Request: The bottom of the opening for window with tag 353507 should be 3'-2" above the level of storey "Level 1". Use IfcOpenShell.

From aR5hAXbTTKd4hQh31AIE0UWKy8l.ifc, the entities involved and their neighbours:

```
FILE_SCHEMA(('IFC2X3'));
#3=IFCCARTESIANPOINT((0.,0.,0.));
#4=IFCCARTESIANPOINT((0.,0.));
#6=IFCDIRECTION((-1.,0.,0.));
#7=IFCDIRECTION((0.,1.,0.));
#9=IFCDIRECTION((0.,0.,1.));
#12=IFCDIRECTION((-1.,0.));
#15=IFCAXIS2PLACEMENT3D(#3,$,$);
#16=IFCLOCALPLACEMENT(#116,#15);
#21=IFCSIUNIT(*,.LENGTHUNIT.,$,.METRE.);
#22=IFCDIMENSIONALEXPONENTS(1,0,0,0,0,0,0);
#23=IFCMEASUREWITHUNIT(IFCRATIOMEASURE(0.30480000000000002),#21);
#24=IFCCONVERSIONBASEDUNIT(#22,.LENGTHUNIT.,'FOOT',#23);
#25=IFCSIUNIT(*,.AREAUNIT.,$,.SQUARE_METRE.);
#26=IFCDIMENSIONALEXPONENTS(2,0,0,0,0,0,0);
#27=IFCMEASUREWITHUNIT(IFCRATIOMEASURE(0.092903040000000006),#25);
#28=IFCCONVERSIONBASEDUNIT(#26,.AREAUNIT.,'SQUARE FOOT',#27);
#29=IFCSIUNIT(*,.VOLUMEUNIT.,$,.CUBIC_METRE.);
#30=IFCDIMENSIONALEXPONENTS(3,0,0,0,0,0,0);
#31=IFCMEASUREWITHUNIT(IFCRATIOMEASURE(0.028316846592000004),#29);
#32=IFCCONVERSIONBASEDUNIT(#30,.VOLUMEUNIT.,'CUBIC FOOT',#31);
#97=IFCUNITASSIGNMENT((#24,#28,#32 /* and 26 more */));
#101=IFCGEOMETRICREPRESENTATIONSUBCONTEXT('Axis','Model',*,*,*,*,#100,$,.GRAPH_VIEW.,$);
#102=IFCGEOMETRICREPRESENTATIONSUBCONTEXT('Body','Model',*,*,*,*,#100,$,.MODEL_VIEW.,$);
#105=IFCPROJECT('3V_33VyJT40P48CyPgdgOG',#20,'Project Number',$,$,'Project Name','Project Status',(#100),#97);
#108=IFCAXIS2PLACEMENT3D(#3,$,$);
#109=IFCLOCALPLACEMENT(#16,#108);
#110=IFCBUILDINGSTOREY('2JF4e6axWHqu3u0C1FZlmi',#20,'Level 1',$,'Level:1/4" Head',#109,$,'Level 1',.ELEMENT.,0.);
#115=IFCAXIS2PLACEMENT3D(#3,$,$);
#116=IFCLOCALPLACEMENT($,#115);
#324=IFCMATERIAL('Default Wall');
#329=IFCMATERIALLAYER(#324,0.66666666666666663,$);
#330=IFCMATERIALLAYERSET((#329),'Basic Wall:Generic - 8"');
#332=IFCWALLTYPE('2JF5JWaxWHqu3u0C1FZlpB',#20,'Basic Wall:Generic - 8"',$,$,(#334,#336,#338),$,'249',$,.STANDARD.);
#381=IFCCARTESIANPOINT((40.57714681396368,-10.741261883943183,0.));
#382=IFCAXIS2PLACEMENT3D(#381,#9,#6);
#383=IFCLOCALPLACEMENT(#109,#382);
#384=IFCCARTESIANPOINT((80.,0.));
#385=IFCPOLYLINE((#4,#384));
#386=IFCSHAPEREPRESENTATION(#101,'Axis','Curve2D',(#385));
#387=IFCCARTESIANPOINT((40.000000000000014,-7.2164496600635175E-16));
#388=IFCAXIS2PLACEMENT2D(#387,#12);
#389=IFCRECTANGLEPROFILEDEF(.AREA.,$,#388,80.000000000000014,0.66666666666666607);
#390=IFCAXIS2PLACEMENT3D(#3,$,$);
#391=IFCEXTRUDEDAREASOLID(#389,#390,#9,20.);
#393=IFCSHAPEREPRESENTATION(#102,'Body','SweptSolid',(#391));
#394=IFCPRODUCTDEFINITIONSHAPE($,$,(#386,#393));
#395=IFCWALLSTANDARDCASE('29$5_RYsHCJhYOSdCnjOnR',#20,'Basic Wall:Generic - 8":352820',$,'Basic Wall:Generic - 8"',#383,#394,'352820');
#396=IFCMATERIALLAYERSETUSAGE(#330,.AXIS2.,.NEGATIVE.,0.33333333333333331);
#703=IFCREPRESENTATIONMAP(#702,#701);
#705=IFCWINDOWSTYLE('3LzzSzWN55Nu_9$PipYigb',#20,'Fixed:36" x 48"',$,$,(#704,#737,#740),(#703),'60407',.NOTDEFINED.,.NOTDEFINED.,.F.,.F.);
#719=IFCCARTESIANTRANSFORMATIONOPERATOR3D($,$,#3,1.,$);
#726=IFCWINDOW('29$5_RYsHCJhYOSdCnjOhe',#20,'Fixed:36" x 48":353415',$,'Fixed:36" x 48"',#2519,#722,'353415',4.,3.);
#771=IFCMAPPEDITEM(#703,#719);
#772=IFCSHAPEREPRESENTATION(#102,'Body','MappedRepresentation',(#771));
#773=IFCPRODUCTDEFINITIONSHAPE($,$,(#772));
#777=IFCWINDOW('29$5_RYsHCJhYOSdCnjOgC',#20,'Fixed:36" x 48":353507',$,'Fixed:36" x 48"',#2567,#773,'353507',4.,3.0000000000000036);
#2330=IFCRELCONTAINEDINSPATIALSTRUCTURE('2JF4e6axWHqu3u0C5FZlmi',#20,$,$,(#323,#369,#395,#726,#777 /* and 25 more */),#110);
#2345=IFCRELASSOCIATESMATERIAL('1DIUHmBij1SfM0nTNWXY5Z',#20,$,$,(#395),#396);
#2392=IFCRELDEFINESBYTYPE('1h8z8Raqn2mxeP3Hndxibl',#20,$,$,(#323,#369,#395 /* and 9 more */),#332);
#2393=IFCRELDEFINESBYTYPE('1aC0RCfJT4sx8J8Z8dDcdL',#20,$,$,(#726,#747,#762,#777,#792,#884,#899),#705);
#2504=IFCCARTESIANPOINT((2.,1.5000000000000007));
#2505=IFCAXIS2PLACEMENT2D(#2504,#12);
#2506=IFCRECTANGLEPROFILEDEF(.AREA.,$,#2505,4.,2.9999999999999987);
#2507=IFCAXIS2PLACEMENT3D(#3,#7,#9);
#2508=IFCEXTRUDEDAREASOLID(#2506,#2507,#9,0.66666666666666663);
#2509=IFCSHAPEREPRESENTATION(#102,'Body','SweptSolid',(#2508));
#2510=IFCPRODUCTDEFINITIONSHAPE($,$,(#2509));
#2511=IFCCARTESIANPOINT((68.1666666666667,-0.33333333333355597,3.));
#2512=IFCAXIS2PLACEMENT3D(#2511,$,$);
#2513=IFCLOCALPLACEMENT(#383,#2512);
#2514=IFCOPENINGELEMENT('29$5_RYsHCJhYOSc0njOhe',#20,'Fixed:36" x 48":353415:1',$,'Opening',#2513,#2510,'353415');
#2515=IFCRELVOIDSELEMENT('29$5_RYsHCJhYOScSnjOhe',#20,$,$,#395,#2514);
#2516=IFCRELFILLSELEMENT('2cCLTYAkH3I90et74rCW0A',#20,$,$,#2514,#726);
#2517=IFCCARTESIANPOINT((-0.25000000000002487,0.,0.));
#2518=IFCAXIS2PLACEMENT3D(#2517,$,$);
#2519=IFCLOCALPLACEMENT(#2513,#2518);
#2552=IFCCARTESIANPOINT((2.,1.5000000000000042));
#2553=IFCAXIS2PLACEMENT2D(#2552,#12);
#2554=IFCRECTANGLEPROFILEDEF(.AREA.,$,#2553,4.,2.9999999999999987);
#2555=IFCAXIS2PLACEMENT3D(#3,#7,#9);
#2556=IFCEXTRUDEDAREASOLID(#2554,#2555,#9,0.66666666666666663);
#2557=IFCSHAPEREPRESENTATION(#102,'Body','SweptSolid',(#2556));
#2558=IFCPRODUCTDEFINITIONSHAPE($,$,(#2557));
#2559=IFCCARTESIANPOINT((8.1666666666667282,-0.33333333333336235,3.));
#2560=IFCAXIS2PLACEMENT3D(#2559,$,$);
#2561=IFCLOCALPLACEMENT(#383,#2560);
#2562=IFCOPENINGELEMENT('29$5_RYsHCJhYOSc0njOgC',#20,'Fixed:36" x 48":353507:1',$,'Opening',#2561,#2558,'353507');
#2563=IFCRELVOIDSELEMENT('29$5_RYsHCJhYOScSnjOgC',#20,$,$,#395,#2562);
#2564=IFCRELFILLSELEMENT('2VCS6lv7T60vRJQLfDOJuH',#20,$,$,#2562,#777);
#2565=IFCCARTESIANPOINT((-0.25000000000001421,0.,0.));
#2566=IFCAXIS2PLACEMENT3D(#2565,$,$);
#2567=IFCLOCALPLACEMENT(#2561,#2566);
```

```python
import numpy as np
import ifcopenshell
import ifcopenshell.api.geometry
import ifcopenshell.geom
import ifcopenshell.util.element
import ifcopenshell.util.placement
import ifcopenshell.util.shape
import ifcopenshell.util.unit

model = ifcopenshell.open("aR5hAXbTTKd4hQh31AIE0UWKy8l.ifc")
unit_scale = ifcopenshell.util.unit.calculate_unit_scale(model)

window = model.by_guid("29$5_RYsHCJhYOSdCnjOgC")
opening = window.FillsVoids[0].RelatingOpeningElement
storey = ifcopenshell.util.element.get_container(window, ifc_class="IfcBuildingStorey")
level = ifcopenshell.util.placement.get_local_placement(storey.ObjectPlacement)[2, 3]

# The opening's origin need not be at the sill, so measure its lowest point.
shape = ifcopenshell.geom.create_shape(ifcopenshell.geom.settings(), opening)
bottom = ifcopenshell.util.shape.get_shape_bottom_elevation(shape, shape.geometry) / unit_scale
dz = level + 38 * 0.0254 / unit_scale - bottom

shift = np.array([0.0, 0.0, dz])
# The window is placed relative to its opening, so it follows when the opening moves.
matrix = ifcopenshell.util.placement.get_local_placement(opening.ObjectPlacement)
matrix[:3, 3] += shift
ifcopenshell.api.geometry.edit_object_placement(
    model, product=opening, matrix=matrix, is_si=False, should_transform_children=True
)

print(f"moved by {dz * unit_scale:+.3f} m")

model.write("aR5hAXbTTKd4hQh31AIE0UWKy8l-out.ifc")
```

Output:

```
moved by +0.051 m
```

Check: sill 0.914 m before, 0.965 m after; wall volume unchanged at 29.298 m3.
